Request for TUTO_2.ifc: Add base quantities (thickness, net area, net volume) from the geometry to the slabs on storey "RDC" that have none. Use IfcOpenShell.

First a look at what the model holds.

```python
import ifcopenshell
import ifcopenshell.util.element
import ifcopenshell.util.unit

model = ifcopenshell.open("TUTO_2.ifc")
print(model.schema)
for unit_type in ("LENGTHUNIT", "AREAUNIT", "VOLUMEUNIT"):
    print(unit_type, ifcopenshell.util.unit.calculate_unit_scale(model, unit_type))
storey = next(s for s in model.by_type("IfcBuildingStorey") if s.Name == "RDC")
slabs = [e for e in ifcopenshell.util.element.get_decomposition(storey) if e.is_a("IfcSlab")]
for e in sorted(slabs, key=lambda e: e.id()):
    print(e.id(), e.is_a(), e.Name, list(ifcopenshell.util.element.get_psets(e, qtos_only=True)), sep=" | ")
```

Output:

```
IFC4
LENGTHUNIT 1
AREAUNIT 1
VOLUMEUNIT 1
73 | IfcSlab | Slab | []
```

```python
import ifcopenshell
import ifcopenshell.api.pset
import ifcopenshell.geom
import ifcopenshell.util.element
import ifcopenshell.util.shape
import ifcopenshell.util.unit

model = ifcopenshell.open("TUTO_2.ifc")
unit_scale = ifcopenshell.util.unit.calculate_unit_scale(model)
area_scale = ifcopenshell.util.unit.calculate_unit_scale(model, "AREAUNIT")
volume_scale = ifcopenshell.util.unit.calculate_unit_scale(model, "VOLUMEUNIT")
settings = ifcopenshell.geom.settings()

storey = next(s for s in model.by_type("IfcBuildingStorey") if s.Name == "RDC")
slabs = [e for e in ifcopenshell.util.element.get_decomposition(storey) if e.is_a("IfcSlab")]

for e in sorted(slabs, key=lambda e: e.id()):
    if ifcopenshell.util.element.get_psets(e, qtos_only=True, should_inherit=False):
        continue
    # Geometry comes back in metres, in the element's own axes.
    shape = ifcopenshell.geom.create_shape(settings, e)
    values = {
        "Width": ifcopenshell.util.shape.get_z(shape.geometry) / unit_scale,
        "NetArea": ifcopenshell.util.shape.get_footprint_area(shape.geometry) / area_scale,
        "NetVolume": ifcopenshell.util.shape.get_volume(shape.geometry) / volume_scale,
    }
    qto = ifcopenshell.api.pset.add_qto(model, product=e, name="Qto_SlabBaseQuantities")
    ifcopenshell.api.pset.edit_qto(model, qto=qto, properties=values)
    print(e.id(), {k: round(v, 3) for k, v in values.items()})

model.write("TUTO_2_v2.ifc")
```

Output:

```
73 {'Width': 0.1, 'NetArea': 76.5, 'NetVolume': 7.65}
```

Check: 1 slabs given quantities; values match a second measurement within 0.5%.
